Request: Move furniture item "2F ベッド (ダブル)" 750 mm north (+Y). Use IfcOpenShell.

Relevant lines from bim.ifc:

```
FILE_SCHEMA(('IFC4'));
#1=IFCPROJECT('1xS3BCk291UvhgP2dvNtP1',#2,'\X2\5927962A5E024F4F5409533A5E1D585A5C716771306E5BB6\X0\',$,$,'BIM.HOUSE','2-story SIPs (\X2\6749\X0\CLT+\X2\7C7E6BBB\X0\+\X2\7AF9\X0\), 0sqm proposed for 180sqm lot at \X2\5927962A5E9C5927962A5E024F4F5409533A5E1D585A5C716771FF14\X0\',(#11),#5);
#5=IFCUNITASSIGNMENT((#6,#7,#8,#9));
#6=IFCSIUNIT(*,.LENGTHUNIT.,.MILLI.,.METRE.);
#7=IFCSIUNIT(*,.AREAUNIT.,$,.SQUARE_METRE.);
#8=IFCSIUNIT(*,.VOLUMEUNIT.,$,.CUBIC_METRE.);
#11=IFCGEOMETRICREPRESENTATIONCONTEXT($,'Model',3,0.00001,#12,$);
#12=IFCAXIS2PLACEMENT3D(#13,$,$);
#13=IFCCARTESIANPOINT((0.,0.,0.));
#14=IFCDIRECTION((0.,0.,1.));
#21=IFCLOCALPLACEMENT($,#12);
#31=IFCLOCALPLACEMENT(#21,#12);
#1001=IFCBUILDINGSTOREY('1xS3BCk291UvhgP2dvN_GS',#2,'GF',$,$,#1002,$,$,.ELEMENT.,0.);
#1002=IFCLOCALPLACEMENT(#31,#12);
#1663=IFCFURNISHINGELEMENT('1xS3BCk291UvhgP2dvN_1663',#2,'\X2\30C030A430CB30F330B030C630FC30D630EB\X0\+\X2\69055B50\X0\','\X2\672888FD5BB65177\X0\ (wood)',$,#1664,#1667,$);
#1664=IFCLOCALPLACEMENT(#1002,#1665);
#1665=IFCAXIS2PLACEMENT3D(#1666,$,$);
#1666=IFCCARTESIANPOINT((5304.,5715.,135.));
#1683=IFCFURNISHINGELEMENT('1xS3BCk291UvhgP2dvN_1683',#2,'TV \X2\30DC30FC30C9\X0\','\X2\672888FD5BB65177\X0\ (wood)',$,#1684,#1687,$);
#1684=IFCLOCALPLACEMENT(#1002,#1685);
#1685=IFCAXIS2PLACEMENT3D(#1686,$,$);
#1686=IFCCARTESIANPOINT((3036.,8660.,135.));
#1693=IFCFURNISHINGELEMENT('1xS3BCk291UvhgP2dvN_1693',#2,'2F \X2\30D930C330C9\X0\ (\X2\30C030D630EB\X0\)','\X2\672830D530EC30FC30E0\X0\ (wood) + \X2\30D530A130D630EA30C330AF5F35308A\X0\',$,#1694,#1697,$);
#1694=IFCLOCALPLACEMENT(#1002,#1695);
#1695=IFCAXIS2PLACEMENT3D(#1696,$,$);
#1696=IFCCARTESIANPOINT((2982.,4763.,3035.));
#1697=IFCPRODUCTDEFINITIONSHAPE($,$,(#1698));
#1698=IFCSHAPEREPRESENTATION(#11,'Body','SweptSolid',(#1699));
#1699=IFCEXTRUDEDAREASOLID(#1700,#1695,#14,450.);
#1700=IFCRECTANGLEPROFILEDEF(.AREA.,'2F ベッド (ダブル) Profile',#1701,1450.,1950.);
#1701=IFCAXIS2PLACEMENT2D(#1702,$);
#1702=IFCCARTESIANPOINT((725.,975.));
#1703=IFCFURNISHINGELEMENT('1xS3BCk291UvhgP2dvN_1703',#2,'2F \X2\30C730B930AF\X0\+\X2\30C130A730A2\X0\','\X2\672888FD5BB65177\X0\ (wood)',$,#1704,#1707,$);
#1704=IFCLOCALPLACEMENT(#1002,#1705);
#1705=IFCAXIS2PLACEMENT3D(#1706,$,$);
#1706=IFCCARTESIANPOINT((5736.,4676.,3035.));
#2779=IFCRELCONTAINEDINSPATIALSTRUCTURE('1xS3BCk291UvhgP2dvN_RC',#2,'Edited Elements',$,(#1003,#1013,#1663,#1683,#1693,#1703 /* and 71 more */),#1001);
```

```python
import ifcopenshell
import ifcopenshell.api.geometry
import ifcopenshell.util.placement
import ifcopenshell.util.unit

model = ifcopenshell.open("bim.ifc")
unit_scale = ifcopenshell.util.unit.calculate_unit_scale(model)

item = model.by_guid("1xS3BCk291UvhgP2dvN_1693")
matrix = ifcopenshell.util.placement.get_local_placement(item.ObjectPlacement)
matrix[1, 3] += 0.75 / unit_scale
ifcopenshell.api.geometry.edit_object_placement(model, product=item, matrix=matrix, is_si=False)

print(ifcopenshell.util.placement.get_local_placement(item.ObjectPlacement).round(3) + 0.0)

model.write("bim_rev.ifc")
```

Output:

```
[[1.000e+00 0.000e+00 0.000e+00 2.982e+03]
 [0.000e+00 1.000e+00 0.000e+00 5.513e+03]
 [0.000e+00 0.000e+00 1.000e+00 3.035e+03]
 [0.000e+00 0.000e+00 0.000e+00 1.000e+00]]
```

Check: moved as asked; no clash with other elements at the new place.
